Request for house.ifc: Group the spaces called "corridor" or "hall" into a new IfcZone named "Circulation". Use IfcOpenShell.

First a look at what the model holds.

```python
import ifcopenshell

model = ifcopenshell.open("house.ifc")
print(model.schema)
seen = {}
for space in model.by_type("IfcSpace"):
    seen[space.LongName] = seen.get(space.LongName, 0) + 1
for name, count in sorted(seen.items(), key=str):
    print(count, "x", name)
print("zones:", [z.Name for z in model.by_type("IfcZone")][:20])
```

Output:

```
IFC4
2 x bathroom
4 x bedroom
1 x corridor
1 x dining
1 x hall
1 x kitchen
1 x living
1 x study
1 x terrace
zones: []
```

```python
import ifcopenshell
import ifcopenshell.api.group
import ifcopenshell.api.root

model = ifcopenshell.open("house.ifc")

names = {"corridor", "hall"}
spaces = [s for s in model.by_type("IfcSpace") if s.LongName in names]

zone = ifcopenshell.api.root.create_entity(model, ifc_class="IfcZone", name="Circulation")
ifcopenshell.api.group.assign_group(model, products=spaces, group=zone)
print(len(spaces), "spaces in", zone.Name)

model.write("house_rev.ifc")
```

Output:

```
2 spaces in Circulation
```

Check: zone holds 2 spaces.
